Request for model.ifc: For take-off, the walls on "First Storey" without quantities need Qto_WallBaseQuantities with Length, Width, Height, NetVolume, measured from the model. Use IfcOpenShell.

First a look at what the model holds.

```python
import ifcopenshell
import ifcopenshell.util.element
import ifcopenshell.util.unit

model = ifcopenshell.open("model.ifc")
print(model.schema)
for unit_type in ("LENGTHUNIT", "AREAUNIT", "VOLUMEUNIT"):
    print(unit_type, ifcopenshell.util.unit.calculate_unit_scale(model, unit_type))
storey = next(s for s in model.by_type("IfcBuildingStorey") if s.Name == "First Storey")
walls = [e for e in ifcopenshell.util.element.get_decomposition(storey) if e.is_a("IfcWall")]
for e in sorted(walls, key=lambda e: e.id()):
    print(e.id(), e.is_a(), e.Name, list(ifcopenshell.util.element.get_psets(e, qtos_only=True)), sep=" | ")
```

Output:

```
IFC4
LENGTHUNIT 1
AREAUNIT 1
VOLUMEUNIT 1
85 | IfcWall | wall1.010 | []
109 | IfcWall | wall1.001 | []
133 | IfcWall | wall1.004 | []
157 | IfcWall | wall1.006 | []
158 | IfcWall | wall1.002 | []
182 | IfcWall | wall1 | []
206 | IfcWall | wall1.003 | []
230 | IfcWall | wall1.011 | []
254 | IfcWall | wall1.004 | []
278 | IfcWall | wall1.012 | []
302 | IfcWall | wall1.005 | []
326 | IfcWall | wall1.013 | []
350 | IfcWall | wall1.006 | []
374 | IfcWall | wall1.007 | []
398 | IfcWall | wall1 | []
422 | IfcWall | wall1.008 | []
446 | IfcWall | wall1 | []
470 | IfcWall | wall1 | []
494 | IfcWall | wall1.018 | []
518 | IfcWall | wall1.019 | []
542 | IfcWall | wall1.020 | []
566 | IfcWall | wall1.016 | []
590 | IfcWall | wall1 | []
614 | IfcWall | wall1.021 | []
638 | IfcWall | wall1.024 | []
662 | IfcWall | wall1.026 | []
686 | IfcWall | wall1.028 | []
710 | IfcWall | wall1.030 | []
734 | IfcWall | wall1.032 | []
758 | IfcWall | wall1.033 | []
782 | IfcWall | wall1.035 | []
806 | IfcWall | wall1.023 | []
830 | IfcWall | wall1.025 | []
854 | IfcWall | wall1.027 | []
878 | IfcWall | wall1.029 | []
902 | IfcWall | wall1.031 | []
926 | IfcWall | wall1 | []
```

```python
import ifcopenshell
import ifcopenshell.api.pset
import ifcopenshell.geom
import ifcopenshell.util.element
import ifcopenshell.util.shape
import ifcopenshell.util.unit

model = ifcopenshell.open("model.ifc")
unit_scale = ifcopenshell.util.unit.calculate_unit_scale(model)
volume_scale = ifcopenshell.util.unit.calculate_unit_scale(model, "VOLUMEUNIT")
settings = ifcopenshell.geom.settings()

storey = next(s for s in model.by_type("IfcBuildingStorey") if s.Name == "First Storey")
walls = [e for e in ifcopenshell.util.element.get_decomposition(storey) if e.is_a("IfcWall")]

for e in sorted(walls, key=lambda e: e.id()):
    if ifcopenshell.util.element.get_psets(e, qtos_only=True, should_inherit=False):
        continue
    # Geometry comes back in metres, in the element's own axes.
    shape = ifcopenshell.geom.create_shape(settings, e)
    values = {
        "Length": ifcopenshell.util.shape.get_x(shape.geometry) / unit_scale,
        "Width": ifcopenshell.util.shape.get_y(shape.geometry) / unit_scale,
        "Height": ifcopenshell.util.shape.get_z(shape.geometry) / unit_scale,
        "NetVolume": ifcopenshell.util.shape.get_volume(shape.geometry) / volume_scale,
    }
    qto = ifcopenshell.api.pset.add_qto(model, product=e, name="Qto_WallBaseQuantities")
    ifcopenshell.api.pset.edit_qto(model, qto=qto, properties=values)
    print(e.id(), {k: round(v, 3) for k, v in values.items()})

model.write("model_updated.ifc")
```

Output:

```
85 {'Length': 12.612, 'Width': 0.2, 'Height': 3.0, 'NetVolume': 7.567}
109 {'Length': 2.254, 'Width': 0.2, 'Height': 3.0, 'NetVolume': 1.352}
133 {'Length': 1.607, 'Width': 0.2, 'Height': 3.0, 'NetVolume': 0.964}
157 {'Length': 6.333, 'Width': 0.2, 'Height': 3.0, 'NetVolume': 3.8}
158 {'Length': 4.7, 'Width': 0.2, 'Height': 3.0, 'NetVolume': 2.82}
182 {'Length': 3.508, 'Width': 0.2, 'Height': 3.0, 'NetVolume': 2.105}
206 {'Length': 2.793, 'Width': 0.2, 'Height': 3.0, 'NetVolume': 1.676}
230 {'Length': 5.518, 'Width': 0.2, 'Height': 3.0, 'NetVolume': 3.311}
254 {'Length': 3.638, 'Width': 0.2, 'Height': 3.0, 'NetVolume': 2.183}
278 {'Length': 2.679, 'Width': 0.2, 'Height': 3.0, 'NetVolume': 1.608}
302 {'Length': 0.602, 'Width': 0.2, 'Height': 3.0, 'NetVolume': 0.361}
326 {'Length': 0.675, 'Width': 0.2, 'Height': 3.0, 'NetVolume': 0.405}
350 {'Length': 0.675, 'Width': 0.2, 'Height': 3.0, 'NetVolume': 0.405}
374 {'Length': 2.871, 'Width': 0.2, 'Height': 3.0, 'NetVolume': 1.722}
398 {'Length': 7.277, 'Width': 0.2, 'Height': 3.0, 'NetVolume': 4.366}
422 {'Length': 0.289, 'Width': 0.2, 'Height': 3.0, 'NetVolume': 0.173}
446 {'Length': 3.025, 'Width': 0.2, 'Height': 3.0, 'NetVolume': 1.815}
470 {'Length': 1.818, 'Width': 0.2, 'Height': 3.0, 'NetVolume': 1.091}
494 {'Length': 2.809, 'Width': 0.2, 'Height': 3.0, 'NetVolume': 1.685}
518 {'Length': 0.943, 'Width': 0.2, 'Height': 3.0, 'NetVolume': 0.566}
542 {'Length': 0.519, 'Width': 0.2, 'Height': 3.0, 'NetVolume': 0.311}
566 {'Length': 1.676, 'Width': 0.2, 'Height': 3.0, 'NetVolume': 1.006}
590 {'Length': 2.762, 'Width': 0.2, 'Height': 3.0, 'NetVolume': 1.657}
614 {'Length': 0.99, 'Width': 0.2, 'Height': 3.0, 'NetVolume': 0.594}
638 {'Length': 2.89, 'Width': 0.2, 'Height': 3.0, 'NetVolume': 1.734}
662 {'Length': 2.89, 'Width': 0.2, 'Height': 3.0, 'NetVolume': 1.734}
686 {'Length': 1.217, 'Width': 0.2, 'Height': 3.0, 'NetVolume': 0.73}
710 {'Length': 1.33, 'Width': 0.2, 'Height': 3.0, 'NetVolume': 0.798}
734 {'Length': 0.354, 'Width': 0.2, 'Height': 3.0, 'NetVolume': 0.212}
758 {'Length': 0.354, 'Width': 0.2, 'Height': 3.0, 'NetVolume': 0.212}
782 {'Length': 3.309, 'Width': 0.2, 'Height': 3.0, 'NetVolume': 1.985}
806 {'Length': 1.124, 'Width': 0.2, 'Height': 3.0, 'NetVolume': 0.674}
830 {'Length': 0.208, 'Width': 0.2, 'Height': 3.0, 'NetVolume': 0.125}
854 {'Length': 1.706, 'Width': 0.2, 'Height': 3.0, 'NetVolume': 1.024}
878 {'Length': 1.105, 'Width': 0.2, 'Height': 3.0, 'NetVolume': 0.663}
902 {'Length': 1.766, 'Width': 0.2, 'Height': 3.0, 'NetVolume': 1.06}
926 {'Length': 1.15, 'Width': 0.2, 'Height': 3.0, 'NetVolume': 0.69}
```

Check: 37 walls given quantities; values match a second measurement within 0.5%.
